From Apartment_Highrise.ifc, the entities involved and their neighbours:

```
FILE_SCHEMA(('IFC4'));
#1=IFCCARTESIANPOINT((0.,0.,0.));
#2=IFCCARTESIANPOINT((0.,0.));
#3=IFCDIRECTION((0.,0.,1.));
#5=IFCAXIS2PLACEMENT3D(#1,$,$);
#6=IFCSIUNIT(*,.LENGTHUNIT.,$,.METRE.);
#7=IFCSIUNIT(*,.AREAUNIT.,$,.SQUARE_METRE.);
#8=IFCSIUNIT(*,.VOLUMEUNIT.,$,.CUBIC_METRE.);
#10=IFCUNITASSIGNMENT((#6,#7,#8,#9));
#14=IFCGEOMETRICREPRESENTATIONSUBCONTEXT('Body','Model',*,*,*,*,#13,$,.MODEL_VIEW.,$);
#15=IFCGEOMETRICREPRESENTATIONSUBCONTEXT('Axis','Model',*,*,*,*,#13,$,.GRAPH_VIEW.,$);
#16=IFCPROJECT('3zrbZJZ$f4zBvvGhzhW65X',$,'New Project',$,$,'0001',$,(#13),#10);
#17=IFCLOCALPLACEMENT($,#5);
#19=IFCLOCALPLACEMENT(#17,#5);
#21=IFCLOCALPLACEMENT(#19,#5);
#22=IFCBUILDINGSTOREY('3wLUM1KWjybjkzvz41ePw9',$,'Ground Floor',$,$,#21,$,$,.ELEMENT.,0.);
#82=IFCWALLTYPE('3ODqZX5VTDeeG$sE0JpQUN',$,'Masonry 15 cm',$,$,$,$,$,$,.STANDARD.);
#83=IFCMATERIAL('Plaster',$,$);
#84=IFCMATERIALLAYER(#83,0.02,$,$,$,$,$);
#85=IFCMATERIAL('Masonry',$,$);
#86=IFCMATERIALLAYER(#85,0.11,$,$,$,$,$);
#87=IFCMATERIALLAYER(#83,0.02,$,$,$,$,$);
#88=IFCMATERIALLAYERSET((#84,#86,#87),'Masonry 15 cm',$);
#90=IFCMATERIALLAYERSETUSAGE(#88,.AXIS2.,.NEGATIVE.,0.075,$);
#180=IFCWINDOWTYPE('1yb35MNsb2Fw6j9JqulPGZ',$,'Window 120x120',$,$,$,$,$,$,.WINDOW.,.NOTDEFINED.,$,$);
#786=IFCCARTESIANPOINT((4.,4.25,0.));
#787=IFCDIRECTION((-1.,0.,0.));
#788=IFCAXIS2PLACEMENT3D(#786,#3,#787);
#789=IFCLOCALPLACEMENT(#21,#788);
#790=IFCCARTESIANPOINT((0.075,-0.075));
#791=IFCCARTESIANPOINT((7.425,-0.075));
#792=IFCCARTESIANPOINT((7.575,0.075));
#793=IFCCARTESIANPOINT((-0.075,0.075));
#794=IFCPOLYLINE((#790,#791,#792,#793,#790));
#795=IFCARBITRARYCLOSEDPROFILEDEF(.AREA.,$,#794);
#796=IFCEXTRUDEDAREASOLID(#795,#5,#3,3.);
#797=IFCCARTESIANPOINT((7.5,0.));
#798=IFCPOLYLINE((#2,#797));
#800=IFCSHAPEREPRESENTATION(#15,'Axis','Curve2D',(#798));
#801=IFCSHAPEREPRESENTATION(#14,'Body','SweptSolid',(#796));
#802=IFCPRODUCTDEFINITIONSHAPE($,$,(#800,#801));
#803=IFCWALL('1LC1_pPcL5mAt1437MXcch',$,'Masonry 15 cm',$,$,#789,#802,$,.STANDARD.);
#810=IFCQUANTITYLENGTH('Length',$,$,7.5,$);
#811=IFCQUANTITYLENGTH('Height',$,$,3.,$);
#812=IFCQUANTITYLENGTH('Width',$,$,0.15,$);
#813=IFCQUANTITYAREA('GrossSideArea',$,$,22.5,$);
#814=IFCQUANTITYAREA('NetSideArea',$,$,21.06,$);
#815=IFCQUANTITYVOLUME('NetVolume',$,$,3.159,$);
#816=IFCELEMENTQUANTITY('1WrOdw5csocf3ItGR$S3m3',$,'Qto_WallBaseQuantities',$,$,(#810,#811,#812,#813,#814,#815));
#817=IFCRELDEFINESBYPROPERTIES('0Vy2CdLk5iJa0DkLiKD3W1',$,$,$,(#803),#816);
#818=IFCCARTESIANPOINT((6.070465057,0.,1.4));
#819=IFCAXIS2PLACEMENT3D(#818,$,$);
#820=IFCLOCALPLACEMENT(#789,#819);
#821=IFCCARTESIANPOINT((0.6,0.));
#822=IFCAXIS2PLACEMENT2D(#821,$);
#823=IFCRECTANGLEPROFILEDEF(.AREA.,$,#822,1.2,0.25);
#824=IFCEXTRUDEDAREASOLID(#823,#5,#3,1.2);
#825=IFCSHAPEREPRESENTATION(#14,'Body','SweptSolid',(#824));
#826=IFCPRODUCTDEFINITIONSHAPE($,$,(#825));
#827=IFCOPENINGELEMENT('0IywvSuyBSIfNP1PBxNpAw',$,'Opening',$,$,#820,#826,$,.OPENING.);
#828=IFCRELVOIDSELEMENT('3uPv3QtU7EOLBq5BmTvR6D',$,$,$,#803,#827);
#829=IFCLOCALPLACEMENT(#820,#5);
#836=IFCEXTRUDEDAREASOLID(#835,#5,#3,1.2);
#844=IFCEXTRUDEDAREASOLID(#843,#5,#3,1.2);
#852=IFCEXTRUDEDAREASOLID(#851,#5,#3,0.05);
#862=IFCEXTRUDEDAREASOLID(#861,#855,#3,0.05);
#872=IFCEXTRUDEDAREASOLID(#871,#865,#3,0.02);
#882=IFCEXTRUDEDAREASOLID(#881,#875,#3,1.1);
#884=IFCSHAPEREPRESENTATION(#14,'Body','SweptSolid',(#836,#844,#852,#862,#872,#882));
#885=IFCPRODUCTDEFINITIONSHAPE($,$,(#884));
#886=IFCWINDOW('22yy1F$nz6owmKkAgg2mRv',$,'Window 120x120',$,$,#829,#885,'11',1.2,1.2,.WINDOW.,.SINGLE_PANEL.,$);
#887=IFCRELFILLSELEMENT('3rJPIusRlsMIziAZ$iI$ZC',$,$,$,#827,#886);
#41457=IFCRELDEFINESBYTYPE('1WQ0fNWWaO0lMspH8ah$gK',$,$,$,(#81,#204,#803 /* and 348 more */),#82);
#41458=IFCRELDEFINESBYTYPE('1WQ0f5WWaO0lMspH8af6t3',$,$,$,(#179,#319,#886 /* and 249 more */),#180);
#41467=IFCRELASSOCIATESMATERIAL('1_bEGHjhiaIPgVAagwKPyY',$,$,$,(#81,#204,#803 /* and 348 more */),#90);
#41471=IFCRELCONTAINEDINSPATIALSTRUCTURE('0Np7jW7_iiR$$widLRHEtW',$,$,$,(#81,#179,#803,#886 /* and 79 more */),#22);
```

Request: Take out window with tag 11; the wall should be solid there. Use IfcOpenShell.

```python
import ifcopenshell
import ifcopenshell.api.feature
import ifcopenshell.api.pset
import ifcopenshell.api.root
import ifcopenshell.geom
import ifcopenshell.util.element
import ifcopenshell.util.shape
import ifcopenshell.util.unit

model = ifcopenshell.open("Apartment_Highrise.ifc")
area_scale = ifcopenshell.util.unit.calculate_unit_scale(model, "AREAUNIT")
volume_scale = ifcopenshell.util.unit.calculate_unit_scale(model, "VOLUMEUNIT")
settings = ifcopenshell.geom.settings()


def volume(element):
    """Net volume in cubic metres, openings subtracted."""
    shape = ifcopenshell.geom.create_shape(settings, element)
    return ifcopenshell.util.shape.get_volume(shape.geometry)


window = model.by_guid("22yy1F$nz6owmKkAgg2mRv")
opening = window.FillsVoids[0].RelatingOpeningElement
wall = opening.VoidsElements[0].RelatingBuildingElement
before = volume(wall)

ifcopenshell.api.root.remove_product(model, product=window)
ifcopenshell.api.feature.remove_feature(model, feature=opening)

after = volume(wall)
thickness = 0.15  # wall thickness in metres

# Update the wall's stored quantities.
qto = model.by_id(ifcopenshell.util.element.get_pset(wall, "Qto_WallBaseQuantities", should_inherit=False)["id"])
ifcopenshell.api.pset.edit_qto(model, qto=qto, properties={
    "NetSideArea": after / thickness / area_scale,
    "NetVolume": after / volume_scale,
})

print(f"wall volume {before:.3f} -> {after:.3f} m3")

model.write("Apartment_Highrise_rev.ifc")
```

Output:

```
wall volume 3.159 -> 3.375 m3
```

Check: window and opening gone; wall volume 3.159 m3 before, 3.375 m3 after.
